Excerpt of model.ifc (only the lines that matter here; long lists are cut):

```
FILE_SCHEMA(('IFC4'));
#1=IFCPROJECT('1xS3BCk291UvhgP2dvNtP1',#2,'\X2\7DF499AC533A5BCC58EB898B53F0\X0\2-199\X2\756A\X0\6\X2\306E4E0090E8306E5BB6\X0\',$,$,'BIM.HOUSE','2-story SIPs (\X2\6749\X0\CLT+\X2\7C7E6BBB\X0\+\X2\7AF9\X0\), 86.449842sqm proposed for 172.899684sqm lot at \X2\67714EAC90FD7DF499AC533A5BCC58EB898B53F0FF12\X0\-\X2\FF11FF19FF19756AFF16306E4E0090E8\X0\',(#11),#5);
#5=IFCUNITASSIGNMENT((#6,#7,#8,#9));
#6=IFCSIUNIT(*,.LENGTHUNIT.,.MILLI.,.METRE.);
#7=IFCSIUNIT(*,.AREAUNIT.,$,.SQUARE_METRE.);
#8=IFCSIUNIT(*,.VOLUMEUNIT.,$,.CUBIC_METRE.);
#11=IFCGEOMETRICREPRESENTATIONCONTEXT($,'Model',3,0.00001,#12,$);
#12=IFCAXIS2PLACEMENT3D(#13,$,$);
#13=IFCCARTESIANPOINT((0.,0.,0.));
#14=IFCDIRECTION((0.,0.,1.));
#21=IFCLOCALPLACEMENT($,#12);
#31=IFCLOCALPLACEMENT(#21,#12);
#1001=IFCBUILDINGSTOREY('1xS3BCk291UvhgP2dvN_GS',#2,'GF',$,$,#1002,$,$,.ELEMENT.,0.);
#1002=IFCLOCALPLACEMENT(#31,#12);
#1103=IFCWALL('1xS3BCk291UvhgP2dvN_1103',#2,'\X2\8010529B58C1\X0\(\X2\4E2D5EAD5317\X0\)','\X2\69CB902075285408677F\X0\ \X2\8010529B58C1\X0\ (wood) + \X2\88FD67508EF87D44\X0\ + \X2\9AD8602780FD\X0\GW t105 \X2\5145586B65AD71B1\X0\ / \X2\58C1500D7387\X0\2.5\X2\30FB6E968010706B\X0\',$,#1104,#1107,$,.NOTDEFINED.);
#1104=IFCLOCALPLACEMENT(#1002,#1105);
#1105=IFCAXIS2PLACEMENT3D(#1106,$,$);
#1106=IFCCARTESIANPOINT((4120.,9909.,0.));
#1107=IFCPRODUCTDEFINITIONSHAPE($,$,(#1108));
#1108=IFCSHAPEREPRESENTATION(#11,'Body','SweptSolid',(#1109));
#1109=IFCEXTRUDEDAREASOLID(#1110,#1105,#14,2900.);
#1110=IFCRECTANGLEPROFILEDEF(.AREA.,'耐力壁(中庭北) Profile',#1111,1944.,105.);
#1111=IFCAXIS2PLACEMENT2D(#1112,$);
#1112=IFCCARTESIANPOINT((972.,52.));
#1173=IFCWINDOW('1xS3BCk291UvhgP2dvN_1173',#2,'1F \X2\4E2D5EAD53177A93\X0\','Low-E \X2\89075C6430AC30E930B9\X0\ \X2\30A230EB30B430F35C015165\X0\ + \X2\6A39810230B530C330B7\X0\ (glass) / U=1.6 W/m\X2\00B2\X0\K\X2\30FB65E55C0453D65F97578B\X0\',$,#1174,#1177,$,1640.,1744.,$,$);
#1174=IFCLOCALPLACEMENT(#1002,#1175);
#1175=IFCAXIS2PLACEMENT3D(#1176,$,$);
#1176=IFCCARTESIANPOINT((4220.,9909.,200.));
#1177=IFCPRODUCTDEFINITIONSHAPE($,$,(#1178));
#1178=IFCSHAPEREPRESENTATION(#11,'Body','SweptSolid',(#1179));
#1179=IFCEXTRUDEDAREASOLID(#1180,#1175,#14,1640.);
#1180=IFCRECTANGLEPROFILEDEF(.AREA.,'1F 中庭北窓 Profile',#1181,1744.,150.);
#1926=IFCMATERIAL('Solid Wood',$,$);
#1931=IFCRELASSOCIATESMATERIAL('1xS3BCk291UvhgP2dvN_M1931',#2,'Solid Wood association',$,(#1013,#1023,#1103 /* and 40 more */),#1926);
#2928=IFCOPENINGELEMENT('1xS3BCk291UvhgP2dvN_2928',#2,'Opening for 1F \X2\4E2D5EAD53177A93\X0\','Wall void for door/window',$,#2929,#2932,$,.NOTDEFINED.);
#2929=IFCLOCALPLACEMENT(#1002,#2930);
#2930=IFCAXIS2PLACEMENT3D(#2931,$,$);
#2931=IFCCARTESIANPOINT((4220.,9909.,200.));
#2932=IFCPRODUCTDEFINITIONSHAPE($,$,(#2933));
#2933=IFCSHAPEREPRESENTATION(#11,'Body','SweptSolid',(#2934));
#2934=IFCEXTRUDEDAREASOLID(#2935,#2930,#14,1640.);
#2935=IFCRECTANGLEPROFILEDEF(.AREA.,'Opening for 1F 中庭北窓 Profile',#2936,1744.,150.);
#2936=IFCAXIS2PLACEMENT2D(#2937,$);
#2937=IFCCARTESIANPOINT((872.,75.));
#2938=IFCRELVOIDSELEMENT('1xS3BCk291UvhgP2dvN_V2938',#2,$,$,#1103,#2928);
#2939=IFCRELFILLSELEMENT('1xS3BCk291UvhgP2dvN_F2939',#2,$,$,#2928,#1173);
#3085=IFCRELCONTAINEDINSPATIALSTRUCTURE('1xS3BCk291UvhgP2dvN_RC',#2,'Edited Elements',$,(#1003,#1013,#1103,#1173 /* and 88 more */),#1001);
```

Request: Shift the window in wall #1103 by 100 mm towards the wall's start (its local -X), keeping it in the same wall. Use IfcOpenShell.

```python
import ifcopenshell
import ifcopenshell.api.geometry
import ifcopenshell.util.placement
import ifcopenshell.util.unit

model = ifcopenshell.open("model.ifc")
unit_scale = ifcopenshell.util.unit.calculate_unit_scale(model)

window = model.by_guid("1xS3BCk291UvhgP2dvN_1173")
opening = window.FillsVoids[0].RelatingOpeningElement
wall = opening.VoidsElements[0].RelatingBuildingElement

wall_matrix = ifcopenshell.util.placement.get_local_placement(wall.ObjectPlacement)
shift = wall_matrix[:3, 0] * -0.1 / unit_scale
before = ifcopenshell.util.placement.get_local_placement(window.ObjectPlacement)[:3, 3].copy()

# The window is not placed relative to its opening, so move both.
for product in (opening, window):
    matrix = ifcopenshell.util.placement.get_local_placement(product.ObjectPlacement)
    matrix[:3, 3] += shift
    ifcopenshell.api.geometry.edit_object_placement(model, product=product, matrix=matrix, is_si=False)

after = ifcopenshell.util.placement.get_local_placement(window.ObjectPlacement)[:3, 3]
print("window moved by", (after - before).round(3) + 0.0)

model.write("model-out.ifc")
```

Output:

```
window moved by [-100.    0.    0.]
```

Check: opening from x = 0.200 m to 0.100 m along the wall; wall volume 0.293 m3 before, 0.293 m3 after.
